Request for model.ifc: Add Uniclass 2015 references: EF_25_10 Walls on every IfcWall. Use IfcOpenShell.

First a look at what the model holds.

```python
import ifcopenshell

model = ifcopenshell.open("model.ifc")
print(model.schema)
print("classifications:", [c.Name for c in model.by_type("IfcClassification")])
for ifc_class in ("IfcDoor", "IfcRoof", "IfcStair", "IfcWall", "IfcWindow"):
    print(ifc_class, len(model.by_type(ifc_class)))
```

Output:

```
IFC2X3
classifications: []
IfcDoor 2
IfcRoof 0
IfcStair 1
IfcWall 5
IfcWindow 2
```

```python
import ifcopenshell
import ifcopenshell.api.classification

model = ifcopenshell.open("model.ifc")

# IFC2X3 requires Source and Edition and has no link from the project to the system.
system = model.create_entity("IfcClassification", Source="NBS", Edition="2015", Name="Uniclass 2015")

codes = {
    "IfcWall": ("EF_25_10", "Walls"),
}
for ifc_class, (code, name) in codes.items():
    products = model.by_type(ifc_class)
    ifcopenshell.api.classification.add_reference(
        model, products=products, classification=system, identification=code, name=name
    )
    print(code, len(products))

model.write("model_rev.ifc")
```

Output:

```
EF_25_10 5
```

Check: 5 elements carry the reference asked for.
